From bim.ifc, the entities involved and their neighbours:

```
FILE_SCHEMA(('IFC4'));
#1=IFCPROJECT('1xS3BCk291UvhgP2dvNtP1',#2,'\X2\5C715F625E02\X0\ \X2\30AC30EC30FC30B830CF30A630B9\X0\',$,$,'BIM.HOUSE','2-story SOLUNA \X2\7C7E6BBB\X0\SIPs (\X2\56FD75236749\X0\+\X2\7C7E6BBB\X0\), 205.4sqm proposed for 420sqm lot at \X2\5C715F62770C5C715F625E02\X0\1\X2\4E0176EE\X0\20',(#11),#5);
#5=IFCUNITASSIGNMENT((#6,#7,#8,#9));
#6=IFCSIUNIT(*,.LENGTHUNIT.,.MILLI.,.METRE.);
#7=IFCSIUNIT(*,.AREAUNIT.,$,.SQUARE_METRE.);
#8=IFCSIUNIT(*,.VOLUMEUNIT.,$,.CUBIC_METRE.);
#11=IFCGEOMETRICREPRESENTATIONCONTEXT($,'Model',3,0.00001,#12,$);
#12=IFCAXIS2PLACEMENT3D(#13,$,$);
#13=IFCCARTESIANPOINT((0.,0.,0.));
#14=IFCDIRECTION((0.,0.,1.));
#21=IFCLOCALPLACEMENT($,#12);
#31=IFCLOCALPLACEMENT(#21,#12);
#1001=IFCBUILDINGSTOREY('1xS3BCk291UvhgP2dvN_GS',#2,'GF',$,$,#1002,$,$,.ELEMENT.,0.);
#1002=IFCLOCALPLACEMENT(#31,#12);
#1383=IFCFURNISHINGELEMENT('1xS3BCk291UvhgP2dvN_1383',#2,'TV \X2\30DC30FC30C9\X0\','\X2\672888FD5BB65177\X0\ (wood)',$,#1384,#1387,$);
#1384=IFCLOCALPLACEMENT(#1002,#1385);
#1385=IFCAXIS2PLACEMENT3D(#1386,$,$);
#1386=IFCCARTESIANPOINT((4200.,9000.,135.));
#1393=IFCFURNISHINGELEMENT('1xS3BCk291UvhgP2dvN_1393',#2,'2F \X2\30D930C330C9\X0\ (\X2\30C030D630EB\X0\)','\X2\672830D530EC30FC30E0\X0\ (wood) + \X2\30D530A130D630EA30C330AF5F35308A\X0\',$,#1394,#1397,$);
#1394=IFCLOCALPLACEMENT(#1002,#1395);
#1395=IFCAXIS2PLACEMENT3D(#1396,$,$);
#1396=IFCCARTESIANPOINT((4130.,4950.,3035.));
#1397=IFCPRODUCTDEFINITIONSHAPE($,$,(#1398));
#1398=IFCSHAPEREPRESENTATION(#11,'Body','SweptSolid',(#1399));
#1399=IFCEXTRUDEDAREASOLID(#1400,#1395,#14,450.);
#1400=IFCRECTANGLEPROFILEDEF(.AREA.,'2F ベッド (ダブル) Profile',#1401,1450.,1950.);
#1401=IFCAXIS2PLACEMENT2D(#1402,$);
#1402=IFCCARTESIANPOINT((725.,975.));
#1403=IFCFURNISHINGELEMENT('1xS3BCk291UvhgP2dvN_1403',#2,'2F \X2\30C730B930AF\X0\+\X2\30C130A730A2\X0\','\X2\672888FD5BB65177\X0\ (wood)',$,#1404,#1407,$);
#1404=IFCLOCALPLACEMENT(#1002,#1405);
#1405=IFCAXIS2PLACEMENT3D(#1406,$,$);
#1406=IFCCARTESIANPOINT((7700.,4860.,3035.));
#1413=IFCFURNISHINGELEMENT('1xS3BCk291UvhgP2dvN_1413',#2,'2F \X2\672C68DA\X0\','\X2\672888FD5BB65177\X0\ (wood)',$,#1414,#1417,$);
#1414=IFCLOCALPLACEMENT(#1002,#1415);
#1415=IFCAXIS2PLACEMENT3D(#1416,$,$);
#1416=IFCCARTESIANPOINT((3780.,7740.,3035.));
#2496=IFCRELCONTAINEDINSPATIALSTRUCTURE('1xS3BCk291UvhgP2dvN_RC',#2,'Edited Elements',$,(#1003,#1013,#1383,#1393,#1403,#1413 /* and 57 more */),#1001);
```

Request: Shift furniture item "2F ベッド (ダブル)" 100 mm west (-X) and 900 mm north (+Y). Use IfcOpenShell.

```python
import ifcopenshell
import ifcopenshell.api.geometry
import ifcopenshell.util.placement
import ifcopenshell.util.unit

model = ifcopenshell.open("bim.ifc")
unit_scale = ifcopenshell.util.unit.calculate_unit_scale(model)

item = model.by_guid("1xS3BCk291UvhgP2dvN_1393")
matrix = ifcopenshell.util.placement.get_local_placement(item.ObjectPlacement)
matrix[0, 3] -= 0.1 / unit_scale
matrix[1, 3] += 0.9 / unit_scale
ifcopenshell.api.geometry.edit_object_placement(model, product=item, matrix=matrix, is_si=False)

print(ifcopenshell.util.placement.get_local_placement(item.ObjectPlacement).round(3) + 0.0)

model.write("bim_edited.ifc")
```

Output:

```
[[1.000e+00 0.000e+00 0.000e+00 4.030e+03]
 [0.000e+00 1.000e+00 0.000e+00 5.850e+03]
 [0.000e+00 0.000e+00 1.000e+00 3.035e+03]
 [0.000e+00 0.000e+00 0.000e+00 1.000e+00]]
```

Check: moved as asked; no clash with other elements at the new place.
